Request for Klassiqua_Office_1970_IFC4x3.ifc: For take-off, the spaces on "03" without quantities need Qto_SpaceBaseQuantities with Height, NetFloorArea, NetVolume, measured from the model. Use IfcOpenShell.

First a look at what the model holds.

```python
import ifcopenshell
import ifcopenshell.util.element
import ifcopenshell.util.unit

model = ifcopenshell.open("Klassiqua_Office_1970_IFC4x3.ifc")
print(model.schema)
for unit_type in ("LENGTHUNIT", "AREAUNIT", "VOLUMEUNIT"):
    print(unit_type, ifcopenshell.util.unit.calculate_unit_scale(model, unit_type))
storey = next(s for s in model.by_type("IfcBuildingStorey") if s.Name == "03")
spaces = [e for e in ifcopenshell.util.element.get_decomposition(storey) if e.is_a("IfcSpace")]
for e in sorted(spaces, key=lambda e: e.id()):
    print(e.id(), e.is_a(), e.Name, list(ifcopenshell.util.element.get_psets(e, qtos_only=True)), sep=" | ")
```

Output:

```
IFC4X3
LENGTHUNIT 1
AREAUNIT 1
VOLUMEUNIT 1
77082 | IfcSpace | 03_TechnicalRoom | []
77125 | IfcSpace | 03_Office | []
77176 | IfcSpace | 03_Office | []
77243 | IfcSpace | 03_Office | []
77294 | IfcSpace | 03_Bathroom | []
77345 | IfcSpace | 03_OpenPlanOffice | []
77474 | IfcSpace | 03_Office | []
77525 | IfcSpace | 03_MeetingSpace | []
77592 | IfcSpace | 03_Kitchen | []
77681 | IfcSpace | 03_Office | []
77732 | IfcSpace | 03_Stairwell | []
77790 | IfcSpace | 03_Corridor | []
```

```python
import ifcopenshell
import ifcopenshell.api.pset
import ifcopenshell.geom
import ifcopenshell.util.element
import ifcopenshell.util.shape
import ifcopenshell.util.unit

model = ifcopenshell.open("Klassiqua_Office_1970_IFC4x3.ifc")
unit_scale = ifcopenshell.util.unit.calculate_unit_scale(model)
area_scale = ifcopenshell.util.unit.calculate_unit_scale(model, "AREAUNIT")
volume_scale = ifcopenshell.util.unit.calculate_unit_scale(model, "VOLUMEUNIT")
settings = ifcopenshell.geom.settings()

storey = next(s for s in model.by_type("IfcBuildingStorey") if s.Name == "03")
spaces = [e for e in ifcopenshell.util.element.get_decomposition(storey) if e.is_a("IfcSpace")]

for e in sorted(spaces, key=lambda e: e.id()):
    if ifcopenshell.util.element.get_psets(e, qtos_only=True, should_inherit=False):
        continue
    # Geometry comes back in metres, in the element's own axes.
    shape = ifcopenshell.geom.create_shape(settings, e)
    values = {
        "Height": ifcopenshell.util.shape.get_z(shape.geometry) / unit_scale,
        "NetFloorArea": ifcopenshell.util.shape.get_footprint_area(shape.geometry) / area_scale,
        "NetVolume": ifcopenshell.util.shape.get_volume(shape.geometry) / volume_scale,
    }
    qto = ifcopenshell.api.pset.add_qto(model, product=e, name="Qto_SpaceBaseQuantities")
    ifcopenshell.api.pset.edit_qto(model, qto=qto, properties=values)
    print(e.id(), {k: round(v, 3) for k, v in values.items()})

model.write("Klassiqua_Office_1970_IFC4x3_updated.ifc")
```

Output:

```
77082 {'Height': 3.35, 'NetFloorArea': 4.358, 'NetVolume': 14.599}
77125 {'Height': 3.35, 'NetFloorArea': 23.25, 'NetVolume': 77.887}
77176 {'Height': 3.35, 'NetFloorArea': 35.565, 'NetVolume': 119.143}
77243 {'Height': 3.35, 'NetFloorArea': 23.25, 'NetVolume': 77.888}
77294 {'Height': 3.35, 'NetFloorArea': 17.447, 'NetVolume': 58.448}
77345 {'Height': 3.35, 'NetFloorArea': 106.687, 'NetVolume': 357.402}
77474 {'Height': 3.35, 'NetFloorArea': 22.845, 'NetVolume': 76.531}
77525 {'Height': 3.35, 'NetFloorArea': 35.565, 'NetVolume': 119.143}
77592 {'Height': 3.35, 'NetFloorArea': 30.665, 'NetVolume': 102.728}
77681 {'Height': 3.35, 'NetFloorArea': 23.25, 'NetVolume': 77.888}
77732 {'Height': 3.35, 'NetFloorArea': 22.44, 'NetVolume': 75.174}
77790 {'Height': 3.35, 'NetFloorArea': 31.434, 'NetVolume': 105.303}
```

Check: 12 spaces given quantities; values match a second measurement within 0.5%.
